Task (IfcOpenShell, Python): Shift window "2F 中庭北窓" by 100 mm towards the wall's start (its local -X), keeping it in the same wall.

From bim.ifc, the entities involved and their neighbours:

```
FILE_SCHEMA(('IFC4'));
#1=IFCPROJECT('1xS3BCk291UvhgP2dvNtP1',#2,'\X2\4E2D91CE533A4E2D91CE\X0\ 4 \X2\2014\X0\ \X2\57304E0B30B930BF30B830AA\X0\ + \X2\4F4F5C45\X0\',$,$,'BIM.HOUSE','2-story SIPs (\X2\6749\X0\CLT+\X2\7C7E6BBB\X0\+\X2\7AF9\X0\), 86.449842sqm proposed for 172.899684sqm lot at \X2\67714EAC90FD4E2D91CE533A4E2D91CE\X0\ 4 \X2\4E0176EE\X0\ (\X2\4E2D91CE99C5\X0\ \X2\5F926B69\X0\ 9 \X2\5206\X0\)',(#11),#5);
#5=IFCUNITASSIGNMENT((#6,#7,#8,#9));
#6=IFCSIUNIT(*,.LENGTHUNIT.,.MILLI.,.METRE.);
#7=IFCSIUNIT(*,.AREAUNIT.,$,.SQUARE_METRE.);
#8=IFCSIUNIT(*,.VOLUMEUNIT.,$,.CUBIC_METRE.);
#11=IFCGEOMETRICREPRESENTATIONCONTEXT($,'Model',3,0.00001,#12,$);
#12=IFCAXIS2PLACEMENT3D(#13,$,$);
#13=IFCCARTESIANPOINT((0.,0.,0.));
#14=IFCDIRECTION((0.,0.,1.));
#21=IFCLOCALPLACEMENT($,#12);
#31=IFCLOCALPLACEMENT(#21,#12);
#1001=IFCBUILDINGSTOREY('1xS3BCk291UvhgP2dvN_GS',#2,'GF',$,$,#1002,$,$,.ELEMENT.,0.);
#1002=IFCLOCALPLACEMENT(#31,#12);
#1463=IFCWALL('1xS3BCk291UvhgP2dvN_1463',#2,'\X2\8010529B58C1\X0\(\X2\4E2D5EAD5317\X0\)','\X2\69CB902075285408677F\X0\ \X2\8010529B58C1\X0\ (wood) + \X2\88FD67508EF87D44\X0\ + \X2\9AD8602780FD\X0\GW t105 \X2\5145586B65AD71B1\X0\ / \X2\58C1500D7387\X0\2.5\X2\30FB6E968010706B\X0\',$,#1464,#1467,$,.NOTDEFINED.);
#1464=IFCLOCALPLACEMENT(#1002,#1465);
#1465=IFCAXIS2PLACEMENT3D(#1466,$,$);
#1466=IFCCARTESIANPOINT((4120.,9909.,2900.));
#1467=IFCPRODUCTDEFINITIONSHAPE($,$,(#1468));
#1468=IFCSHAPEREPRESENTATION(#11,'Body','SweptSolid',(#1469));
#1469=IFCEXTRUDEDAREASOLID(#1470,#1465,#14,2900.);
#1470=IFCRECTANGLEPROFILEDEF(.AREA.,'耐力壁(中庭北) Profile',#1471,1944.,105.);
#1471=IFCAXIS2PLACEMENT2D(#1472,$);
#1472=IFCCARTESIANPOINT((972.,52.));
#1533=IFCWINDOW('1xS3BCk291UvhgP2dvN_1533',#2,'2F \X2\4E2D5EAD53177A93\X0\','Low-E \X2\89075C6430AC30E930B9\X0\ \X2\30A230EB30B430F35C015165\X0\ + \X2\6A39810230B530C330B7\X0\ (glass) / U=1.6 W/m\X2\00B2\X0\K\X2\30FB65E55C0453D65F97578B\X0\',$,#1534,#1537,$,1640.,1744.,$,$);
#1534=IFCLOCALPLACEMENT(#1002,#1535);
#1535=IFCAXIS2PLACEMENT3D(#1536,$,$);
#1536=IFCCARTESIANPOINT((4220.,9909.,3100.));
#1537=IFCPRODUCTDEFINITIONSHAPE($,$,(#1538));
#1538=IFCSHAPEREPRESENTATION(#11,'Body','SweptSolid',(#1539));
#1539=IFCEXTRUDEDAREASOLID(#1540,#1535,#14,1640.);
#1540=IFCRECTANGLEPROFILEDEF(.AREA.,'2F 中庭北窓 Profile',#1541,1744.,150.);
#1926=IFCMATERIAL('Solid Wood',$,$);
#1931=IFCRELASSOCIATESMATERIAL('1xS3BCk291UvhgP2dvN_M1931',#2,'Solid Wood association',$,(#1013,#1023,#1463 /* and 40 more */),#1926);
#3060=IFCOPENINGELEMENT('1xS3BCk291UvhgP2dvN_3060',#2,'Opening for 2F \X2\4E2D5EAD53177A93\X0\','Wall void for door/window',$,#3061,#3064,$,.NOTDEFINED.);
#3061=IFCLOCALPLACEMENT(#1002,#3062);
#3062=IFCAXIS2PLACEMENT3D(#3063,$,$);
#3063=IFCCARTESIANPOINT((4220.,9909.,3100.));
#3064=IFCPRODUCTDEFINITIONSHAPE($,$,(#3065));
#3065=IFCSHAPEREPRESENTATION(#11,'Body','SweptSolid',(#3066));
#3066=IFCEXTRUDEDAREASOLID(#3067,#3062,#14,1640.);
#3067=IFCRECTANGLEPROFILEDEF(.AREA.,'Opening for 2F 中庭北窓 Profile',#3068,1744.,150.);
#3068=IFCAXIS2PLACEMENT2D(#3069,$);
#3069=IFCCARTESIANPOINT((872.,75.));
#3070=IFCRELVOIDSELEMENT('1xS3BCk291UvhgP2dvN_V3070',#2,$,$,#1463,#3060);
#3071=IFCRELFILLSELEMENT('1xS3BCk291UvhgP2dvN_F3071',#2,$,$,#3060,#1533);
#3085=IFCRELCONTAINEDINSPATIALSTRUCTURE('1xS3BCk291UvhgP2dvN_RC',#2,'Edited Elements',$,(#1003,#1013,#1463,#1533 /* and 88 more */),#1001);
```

```python
import ifcopenshell
import ifcopenshell.api.geometry
import ifcopenshell.util.placement

model = ifcopenshell.open("bim.ifc")

window = model.by_guid("1xS3BCk291UvhgP2dvN_1533")
opening = window.FillsVoids[0].RelatingOpeningElement
wall = opening.VoidsElements[0].RelatingBuildingElement

wall_matrix = ifcopenshell.util.placement.get_local_placement(wall.ObjectPlacement)
shift = wall_matrix[:3, 0] * -100.0
before = ifcopenshell.util.placement.get_local_placement(window.ObjectPlacement)[:3, 3].copy()

# The window is not placed relative to its opening, so move both.
for product in (opening, window):
    matrix = ifcopenshell.util.placement.get_local_placement(product.ObjectPlacement)
    matrix[:3, 3] += shift
    ifcopenshell.api.geometry.edit_object_placement(model, product=product, matrix=matrix, is_si=False)

after = ifcopenshell.util.placement.get_local_placement(window.ObjectPlacement)[:3, 3]
print("window moved by", (after - before).round(3) + 0.0)

model.write("bim_updated.ifc")
```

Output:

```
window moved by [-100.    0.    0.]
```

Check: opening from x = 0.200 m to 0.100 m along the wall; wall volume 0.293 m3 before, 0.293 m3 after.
